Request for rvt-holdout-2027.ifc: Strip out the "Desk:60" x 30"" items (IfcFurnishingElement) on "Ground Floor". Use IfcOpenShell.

First a look at what the model holds.

```python
import ifcopenshell
import ifcopenshell.util.element

model = ifcopenshell.open("rvt-holdout-2027.ifc")
print(model.schema)
storey = next(s for s in model.by_type("IfcBuildingStorey") if s.Name == "Ground Floor")
furniture = [e for e in ifcopenshell.util.element.get_decomposition(storey) if e.is_a("IfcFurnishingElement")]
seen = {}
for e in furniture:
    element_type = ifcopenshell.util.element.get_type(e)
    name = element_type.Name if element_type not in (None, e) else None
    seen[name] = seen.get(name, 0) + 1
for name, count in sorted(seen.items(), key=str):
    print(count, "x", name)
```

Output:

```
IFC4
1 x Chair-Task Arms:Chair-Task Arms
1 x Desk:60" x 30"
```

```python
import ifcopenshell
import ifcopenshell.api.root
import ifcopenshell.util.element

model = ifcopenshell.open("rvt-holdout-2027.ifc")

storey = next(s for s in model.by_type("IfcBuildingStorey") if s.Name == "Ground Floor")
furniture = [e for e in ifcopenshell.util.element.get_decomposition(storey) if e.is_a("IfcFurnishingElement")]
targets = [e for e in furniture if (t := ifcopenshell.util.element.get_type(e)) not in (None, e) and t.Name == 'Desk:60" x 30"']

for e in targets:
    ifcopenshell.api.root.remove_product(model, product=e)
print(len(targets), "removed")

model.write("rvt-holdout-2027_edited.ifc")
```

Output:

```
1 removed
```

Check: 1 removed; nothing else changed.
